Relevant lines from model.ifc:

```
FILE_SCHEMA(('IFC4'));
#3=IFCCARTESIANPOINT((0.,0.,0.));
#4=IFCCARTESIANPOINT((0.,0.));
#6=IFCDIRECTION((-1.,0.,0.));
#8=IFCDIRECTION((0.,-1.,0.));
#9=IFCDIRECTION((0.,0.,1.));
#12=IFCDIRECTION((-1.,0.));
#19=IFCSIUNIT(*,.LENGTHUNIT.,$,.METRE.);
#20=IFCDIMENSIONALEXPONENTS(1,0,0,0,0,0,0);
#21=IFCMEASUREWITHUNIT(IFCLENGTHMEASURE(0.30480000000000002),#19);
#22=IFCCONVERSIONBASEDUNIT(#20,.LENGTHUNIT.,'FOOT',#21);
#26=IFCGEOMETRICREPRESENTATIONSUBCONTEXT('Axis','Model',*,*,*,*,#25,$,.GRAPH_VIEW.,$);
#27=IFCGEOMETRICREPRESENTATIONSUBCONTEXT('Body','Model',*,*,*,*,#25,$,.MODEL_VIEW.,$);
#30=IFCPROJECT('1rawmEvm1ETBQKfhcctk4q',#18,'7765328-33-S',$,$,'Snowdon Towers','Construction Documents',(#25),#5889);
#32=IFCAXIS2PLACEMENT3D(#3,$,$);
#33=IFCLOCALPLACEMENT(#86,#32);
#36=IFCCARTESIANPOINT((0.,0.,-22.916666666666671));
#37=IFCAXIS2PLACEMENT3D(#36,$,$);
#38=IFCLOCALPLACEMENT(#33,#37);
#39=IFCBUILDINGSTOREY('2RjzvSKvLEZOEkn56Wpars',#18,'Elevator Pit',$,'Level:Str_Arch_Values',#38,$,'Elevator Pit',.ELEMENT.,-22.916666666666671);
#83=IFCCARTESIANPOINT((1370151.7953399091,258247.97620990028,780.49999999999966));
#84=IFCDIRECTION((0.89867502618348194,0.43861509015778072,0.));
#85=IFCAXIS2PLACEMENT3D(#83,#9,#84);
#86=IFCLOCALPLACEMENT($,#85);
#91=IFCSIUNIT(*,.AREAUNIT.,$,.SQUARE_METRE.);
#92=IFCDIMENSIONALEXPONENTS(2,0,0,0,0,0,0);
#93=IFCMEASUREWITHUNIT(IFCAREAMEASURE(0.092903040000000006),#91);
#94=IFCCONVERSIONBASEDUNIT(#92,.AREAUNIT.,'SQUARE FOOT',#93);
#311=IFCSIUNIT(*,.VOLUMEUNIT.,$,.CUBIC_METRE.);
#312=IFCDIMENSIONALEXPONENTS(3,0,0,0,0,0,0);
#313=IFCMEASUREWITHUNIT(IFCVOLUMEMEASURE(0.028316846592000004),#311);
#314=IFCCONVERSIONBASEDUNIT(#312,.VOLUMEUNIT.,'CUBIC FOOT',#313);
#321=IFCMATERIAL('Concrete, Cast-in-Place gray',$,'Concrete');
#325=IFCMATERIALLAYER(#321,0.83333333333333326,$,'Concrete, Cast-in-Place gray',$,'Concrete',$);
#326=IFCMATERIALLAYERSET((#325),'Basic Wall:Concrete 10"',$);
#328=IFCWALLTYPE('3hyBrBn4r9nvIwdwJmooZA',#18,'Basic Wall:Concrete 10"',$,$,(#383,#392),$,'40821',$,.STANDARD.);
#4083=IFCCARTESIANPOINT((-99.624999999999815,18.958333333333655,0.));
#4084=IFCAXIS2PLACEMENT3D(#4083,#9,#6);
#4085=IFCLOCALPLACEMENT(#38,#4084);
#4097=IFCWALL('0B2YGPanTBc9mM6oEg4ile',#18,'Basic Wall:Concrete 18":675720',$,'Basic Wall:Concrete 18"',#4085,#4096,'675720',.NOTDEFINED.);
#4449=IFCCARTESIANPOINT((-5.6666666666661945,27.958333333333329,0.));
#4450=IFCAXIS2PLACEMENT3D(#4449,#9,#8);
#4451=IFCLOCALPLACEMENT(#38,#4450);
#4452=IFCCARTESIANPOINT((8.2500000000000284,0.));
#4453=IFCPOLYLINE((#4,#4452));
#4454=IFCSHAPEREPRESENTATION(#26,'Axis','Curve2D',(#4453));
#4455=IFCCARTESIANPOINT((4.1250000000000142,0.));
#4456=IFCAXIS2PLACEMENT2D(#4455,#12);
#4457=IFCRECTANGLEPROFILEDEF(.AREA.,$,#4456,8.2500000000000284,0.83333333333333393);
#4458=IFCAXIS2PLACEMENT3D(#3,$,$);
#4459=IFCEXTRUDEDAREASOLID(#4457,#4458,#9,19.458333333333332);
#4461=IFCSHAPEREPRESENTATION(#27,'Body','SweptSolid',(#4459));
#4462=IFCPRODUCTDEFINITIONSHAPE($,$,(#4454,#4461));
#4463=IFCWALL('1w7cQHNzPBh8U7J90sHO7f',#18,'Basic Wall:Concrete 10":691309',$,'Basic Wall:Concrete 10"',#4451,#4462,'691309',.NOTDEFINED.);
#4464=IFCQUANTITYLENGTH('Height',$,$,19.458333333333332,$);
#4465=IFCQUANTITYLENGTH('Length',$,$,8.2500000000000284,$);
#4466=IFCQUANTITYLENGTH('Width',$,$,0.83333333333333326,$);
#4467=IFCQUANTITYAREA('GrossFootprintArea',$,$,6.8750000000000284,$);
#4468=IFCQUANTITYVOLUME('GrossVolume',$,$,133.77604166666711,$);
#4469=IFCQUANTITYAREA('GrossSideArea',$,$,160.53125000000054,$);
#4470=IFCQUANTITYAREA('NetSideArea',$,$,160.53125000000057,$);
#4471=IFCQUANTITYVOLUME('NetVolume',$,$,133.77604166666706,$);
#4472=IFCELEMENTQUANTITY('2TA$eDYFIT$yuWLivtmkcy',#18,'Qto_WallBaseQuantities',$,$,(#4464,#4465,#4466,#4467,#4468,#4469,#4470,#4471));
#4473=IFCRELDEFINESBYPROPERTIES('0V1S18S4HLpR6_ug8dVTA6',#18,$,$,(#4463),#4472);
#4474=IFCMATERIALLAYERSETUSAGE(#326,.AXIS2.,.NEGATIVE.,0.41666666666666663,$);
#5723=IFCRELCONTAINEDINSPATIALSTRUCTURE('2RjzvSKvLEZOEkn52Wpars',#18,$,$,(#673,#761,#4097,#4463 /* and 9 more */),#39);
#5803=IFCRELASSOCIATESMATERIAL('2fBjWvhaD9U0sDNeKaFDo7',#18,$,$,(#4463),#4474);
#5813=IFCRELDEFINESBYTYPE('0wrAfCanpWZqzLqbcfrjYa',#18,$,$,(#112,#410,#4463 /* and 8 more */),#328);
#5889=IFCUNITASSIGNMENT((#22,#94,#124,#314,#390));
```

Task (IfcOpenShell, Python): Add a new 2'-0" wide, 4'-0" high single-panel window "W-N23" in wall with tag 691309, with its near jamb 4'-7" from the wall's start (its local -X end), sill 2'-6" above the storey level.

```python
import numpy as np
import ifcopenshell
import ifcopenshell.api.feature
import ifcopenshell.api.geometry
import ifcopenshell.api.pset
import ifcopenshell.api.root
import ifcopenshell.api.spatial
import ifcopenshell.geom
import ifcopenshell.util.element
import ifcopenshell.util.placement
import ifcopenshell.util.representation
import ifcopenshell.util.shape
import ifcopenshell.util.unit

model = ifcopenshell.open("model.ifc")
unit_scale = ifcopenshell.util.unit.calculate_unit_scale(model)
area_scale = ifcopenshell.util.unit.calculate_unit_scale(model, "AREAUNIT")
volume_scale = ifcopenshell.util.unit.calculate_unit_scale(model, "VOLUMEUNIT")
settings = ifcopenshell.geom.settings()


def volume(element):
    """Net volume in cubic metres, openings subtracted."""
    shape = ifcopenshell.geom.create_shape(settings, element)
    return ifcopenshell.util.shape.get_volume(shape.geometry)


wall = model.by_guid("1w7cQHNzPBh8U7J90sHO7f")
storey = ifcopenshell.util.element.get_container(wall, ifc_class="IfcBuildingStorey")
context = ifcopenshell.util.representation.get_context(model, "Model", "Body", "MODEL_VIEW")
before = volume(wall)

width, height, from_end, sill = 0.6096, 1.2192, 1.397, 0.762  # metres

# The wall runs along its own X axis, and the end named is its -X end.
wall_shape = ifcopenshell.geom.create_shape(settings, wall)
x, y, z = ifcopenshell.util.shape.get_vertices(wall_shape.geometry).T
start = x.min() + from_end
face, thickness = float(y.min()), float(y.max() - y.min())
wall_matrix = ifcopenshell.util.placement.get_local_placement(wall.ObjectPlacement)
level = ifcopenshell.util.placement.get_local_placement(storey.ObjectPlacement)[2, 3]


def in_wall(x, y):
    """Placement at x, y metres in the wall's axes, at sill height."""
    matrix = wall_matrix.copy()
    matrix[:, 3] = wall_matrix @ np.array([x / unit_scale, y / unit_scale, 0.0, 1.0])
    matrix[2, 3] = level + sill / unit_scale
    return matrix


# Opening: a box that overshoots both wall faces by 50 mm.
opening = ifcopenshell.api.root.create_entity(model, ifc_class="IfcOpeningElement", predefined_type="OPENING")
box = ifcopenshell.api.geometry.add_wall_representation(
    model, context=context, length=width, height=height, thickness=thickness + 0.1
)
ifcopenshell.api.geometry.assign_representation(model, product=opening, representation=box)
ifcopenshell.api.geometry.edit_object_placement(model, product=opening, matrix=in_wall(start, face - 0.05), is_si=False)
ifcopenshell.api.feature.add_feature(model, feature=opening, element=wall)

window = ifcopenshell.api.root.create_entity(model, ifc_class="IfcWindow", name="W-N23", predefined_type="WINDOW")
window.OverallWidth, window.OverallHeight = width / unit_scale, height / unit_scale
window.PartitioningType = "SINGLE_PANEL"
body = ifcopenshell.api.geometry.add_window_representation(
    model,
    context=context,
    overall_width=window.OverallWidth,
    overall_height=window.OverallHeight,
    partition_type="SINGLE_PANEL",
)
ifcopenshell.api.geometry.assign_representation(model, product=window, representation=body)
ifcopenshell.api.spatial.assign_container(model, products=[window], relating_structure=storey)
ifcopenshell.api.feature.add_filling(model, opening=opening, element=window)

# Centre the window in the wall's thickness.
ifcopenshell.api.geometry.edit_object_placement(model, product=window, matrix=in_wall(start, face), is_si=False)
window_shape = ifcopenshell.geom.create_shape(settings, window)
depth = ifcopenshell.util.shape.get_vertices(window_shape.geometry)[:, 1]
offset = face + thickness / 2 - (depth.min() + depth.max()) / 2
ifcopenshell.api.geometry.edit_object_placement(model, product=window, matrix=in_wall(start, offset), is_si=False)

after = volume(wall)

# Update the wall's stored quantities.
qto = model.by_id(ifcopenshell.util.element.get_pset(wall, "Qto_WallBaseQuantities", should_inherit=False)["id"])
ifcopenshell.api.pset.edit_qto(model, qto=qto, properties={
    "NetSideArea": after / thickness / area_scale,
    "NetVolume": after / volume_scale,
})

print(f"wall volume {before:.3f} -> {after:.3f} m3")

model.write("model_rev.ifc")
```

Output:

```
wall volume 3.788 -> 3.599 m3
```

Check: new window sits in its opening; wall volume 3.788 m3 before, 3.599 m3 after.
